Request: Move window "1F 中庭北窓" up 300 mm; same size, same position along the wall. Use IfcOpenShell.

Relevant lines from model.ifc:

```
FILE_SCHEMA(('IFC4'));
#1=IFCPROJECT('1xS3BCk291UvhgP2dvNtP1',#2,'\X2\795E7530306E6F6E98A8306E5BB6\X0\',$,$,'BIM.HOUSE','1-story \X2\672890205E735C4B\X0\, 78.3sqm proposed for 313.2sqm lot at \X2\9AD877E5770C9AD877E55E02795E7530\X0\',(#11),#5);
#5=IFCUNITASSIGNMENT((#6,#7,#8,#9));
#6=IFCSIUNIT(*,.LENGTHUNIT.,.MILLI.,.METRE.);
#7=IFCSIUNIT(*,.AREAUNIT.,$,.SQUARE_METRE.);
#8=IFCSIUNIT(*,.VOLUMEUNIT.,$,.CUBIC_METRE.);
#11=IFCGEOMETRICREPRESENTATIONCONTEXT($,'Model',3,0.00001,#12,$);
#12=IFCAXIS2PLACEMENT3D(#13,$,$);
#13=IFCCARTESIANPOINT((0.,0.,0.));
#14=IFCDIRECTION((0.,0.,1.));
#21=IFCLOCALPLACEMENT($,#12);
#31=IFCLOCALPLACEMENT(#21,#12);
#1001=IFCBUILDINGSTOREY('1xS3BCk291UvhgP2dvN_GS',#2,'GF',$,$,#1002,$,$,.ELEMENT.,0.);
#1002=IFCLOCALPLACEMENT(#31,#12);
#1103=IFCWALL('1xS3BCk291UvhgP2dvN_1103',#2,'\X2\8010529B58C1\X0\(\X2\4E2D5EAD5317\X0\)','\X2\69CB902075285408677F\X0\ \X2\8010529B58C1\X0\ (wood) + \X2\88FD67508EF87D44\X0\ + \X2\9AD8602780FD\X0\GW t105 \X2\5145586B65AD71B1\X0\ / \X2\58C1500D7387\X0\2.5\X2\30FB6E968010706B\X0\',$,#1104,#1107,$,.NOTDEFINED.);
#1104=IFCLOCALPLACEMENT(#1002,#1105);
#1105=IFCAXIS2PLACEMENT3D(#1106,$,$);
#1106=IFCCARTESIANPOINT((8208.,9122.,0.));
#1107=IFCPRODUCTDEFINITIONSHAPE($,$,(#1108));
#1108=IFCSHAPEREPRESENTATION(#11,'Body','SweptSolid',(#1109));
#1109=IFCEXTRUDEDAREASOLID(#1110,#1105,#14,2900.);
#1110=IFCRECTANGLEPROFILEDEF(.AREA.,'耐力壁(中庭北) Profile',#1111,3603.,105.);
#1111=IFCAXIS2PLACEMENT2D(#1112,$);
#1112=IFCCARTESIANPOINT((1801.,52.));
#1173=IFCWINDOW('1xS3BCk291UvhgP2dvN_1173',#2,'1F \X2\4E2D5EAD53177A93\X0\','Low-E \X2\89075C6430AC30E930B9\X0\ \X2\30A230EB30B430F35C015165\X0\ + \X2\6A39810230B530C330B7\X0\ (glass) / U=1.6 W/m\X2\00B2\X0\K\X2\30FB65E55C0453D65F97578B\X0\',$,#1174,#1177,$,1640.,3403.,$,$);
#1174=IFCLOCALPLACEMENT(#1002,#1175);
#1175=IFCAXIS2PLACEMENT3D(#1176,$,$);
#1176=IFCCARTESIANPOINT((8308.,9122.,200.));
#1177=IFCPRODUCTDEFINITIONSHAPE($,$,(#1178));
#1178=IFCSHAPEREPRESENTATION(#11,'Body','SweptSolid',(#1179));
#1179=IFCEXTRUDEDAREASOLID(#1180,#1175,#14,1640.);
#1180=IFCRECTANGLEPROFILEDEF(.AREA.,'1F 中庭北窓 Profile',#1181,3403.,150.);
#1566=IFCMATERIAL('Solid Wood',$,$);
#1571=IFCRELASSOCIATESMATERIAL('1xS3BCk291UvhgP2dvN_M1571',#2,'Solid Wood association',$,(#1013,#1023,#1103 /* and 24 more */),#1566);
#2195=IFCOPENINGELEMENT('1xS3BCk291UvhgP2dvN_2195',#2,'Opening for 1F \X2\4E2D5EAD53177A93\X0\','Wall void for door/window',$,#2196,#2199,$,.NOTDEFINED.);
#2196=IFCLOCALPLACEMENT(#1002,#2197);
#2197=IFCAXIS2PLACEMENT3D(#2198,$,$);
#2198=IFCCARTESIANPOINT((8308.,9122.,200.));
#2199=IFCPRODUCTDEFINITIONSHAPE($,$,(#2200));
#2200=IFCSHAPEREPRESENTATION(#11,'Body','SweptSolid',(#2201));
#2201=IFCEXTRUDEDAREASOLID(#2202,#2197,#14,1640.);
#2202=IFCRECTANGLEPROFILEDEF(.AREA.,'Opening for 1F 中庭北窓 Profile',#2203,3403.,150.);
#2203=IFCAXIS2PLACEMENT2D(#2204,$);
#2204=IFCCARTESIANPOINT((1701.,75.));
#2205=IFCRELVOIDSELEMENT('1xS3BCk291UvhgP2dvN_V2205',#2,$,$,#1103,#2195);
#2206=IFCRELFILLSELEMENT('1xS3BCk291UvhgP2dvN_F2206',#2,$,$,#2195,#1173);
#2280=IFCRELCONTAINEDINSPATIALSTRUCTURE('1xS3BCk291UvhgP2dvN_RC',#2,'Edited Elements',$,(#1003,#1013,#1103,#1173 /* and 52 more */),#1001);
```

```python
import numpy as np
import ifcopenshell
import ifcopenshell.api.geometry
import ifcopenshell.util.placement
import ifcopenshell.util.unit

model = ifcopenshell.open("model.ifc")
unit_scale = ifcopenshell.util.unit.calculate_unit_scale(model)

window = model.by_guid("1xS3BCk291UvhgP2dvN_1173")
opening = window.FillsVoids[0].RelatingOpeningElement
dz = 300.0

shift = np.array([0.0, 0.0, dz])
# The window is not placed relative to its opening, so move both.
for product in (opening, window):
    matrix = ifcopenshell.util.placement.get_local_placement(product.ObjectPlacement)
    matrix[:3, 3] += shift
    ifcopenshell.api.geometry.edit_object_placement(model, product=product, matrix=matrix, is_si=False)

print(f"moved by {dz * unit_scale:+.3f} m")

model.write("model_v2.ifc")
```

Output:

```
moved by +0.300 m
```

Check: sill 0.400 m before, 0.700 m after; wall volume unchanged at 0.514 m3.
